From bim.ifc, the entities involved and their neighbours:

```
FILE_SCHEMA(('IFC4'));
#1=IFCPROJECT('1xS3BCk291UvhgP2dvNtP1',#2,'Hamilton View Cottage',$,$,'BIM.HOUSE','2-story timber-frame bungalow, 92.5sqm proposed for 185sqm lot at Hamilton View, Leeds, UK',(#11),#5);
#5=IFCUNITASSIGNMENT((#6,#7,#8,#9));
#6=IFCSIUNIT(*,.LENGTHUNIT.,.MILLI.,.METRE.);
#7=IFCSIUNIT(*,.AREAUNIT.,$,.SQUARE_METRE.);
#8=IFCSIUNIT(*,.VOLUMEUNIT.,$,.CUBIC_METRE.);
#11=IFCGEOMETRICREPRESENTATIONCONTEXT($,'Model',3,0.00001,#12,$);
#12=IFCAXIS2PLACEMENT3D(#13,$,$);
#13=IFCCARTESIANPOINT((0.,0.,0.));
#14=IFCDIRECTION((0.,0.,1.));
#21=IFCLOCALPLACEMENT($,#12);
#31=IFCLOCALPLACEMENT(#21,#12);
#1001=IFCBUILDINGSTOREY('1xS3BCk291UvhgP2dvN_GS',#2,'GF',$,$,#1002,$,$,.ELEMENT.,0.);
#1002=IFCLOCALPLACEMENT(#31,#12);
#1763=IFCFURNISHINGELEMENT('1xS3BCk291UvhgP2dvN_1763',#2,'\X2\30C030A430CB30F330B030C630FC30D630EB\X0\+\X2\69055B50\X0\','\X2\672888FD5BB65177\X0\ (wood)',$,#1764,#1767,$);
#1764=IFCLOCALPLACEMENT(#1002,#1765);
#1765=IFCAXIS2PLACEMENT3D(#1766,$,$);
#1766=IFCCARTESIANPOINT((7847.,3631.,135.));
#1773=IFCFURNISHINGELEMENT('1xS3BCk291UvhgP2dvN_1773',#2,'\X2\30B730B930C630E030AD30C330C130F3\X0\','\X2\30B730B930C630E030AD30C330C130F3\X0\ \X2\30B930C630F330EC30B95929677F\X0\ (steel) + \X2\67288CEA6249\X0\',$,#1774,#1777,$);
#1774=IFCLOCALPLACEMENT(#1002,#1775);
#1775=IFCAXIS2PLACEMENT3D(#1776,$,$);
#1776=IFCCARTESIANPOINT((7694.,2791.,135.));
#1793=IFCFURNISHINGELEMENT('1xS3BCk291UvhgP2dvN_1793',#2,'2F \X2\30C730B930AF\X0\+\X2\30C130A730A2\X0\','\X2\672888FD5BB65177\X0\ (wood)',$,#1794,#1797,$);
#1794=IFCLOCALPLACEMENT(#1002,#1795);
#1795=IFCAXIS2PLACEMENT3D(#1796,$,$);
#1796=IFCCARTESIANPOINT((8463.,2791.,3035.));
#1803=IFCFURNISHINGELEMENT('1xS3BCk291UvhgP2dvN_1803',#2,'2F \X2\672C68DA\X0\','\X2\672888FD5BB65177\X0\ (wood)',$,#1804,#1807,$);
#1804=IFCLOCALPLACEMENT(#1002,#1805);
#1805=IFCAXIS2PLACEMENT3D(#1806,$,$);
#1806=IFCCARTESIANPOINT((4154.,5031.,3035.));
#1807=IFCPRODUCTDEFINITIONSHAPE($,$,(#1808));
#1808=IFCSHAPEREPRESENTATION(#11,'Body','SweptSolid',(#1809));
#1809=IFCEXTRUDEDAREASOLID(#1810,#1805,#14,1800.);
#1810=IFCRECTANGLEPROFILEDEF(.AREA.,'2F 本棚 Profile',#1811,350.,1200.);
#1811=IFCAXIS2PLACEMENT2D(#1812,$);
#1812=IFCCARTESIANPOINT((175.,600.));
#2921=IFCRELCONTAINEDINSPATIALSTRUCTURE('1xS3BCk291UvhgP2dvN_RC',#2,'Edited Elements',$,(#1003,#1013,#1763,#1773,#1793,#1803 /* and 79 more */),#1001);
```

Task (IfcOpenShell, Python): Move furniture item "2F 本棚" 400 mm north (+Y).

```python
import ifcopenshell
import ifcopenshell.api.geometry
import ifcopenshell.util.placement
import ifcopenshell.util.unit

model = ifcopenshell.open("bim.ifc")
unit_scale = ifcopenshell.util.unit.calculate_unit_scale(model)

item = model.by_guid("1xS3BCk291UvhgP2dvN_1803")
matrix = ifcopenshell.util.placement.get_local_placement(item.ObjectPlacement)
matrix[1, 3] += 0.4 / unit_scale
ifcopenshell.api.geometry.edit_object_placement(model, product=item, matrix=matrix, is_si=False)

print(ifcopenshell.util.placement.get_local_placement(item.ObjectPlacement).round(3) + 0.0)

model.write("bim_rev.ifc")
```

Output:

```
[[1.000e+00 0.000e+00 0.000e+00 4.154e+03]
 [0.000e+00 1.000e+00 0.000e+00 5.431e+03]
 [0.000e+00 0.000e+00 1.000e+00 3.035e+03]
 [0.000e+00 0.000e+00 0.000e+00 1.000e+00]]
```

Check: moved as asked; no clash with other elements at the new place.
